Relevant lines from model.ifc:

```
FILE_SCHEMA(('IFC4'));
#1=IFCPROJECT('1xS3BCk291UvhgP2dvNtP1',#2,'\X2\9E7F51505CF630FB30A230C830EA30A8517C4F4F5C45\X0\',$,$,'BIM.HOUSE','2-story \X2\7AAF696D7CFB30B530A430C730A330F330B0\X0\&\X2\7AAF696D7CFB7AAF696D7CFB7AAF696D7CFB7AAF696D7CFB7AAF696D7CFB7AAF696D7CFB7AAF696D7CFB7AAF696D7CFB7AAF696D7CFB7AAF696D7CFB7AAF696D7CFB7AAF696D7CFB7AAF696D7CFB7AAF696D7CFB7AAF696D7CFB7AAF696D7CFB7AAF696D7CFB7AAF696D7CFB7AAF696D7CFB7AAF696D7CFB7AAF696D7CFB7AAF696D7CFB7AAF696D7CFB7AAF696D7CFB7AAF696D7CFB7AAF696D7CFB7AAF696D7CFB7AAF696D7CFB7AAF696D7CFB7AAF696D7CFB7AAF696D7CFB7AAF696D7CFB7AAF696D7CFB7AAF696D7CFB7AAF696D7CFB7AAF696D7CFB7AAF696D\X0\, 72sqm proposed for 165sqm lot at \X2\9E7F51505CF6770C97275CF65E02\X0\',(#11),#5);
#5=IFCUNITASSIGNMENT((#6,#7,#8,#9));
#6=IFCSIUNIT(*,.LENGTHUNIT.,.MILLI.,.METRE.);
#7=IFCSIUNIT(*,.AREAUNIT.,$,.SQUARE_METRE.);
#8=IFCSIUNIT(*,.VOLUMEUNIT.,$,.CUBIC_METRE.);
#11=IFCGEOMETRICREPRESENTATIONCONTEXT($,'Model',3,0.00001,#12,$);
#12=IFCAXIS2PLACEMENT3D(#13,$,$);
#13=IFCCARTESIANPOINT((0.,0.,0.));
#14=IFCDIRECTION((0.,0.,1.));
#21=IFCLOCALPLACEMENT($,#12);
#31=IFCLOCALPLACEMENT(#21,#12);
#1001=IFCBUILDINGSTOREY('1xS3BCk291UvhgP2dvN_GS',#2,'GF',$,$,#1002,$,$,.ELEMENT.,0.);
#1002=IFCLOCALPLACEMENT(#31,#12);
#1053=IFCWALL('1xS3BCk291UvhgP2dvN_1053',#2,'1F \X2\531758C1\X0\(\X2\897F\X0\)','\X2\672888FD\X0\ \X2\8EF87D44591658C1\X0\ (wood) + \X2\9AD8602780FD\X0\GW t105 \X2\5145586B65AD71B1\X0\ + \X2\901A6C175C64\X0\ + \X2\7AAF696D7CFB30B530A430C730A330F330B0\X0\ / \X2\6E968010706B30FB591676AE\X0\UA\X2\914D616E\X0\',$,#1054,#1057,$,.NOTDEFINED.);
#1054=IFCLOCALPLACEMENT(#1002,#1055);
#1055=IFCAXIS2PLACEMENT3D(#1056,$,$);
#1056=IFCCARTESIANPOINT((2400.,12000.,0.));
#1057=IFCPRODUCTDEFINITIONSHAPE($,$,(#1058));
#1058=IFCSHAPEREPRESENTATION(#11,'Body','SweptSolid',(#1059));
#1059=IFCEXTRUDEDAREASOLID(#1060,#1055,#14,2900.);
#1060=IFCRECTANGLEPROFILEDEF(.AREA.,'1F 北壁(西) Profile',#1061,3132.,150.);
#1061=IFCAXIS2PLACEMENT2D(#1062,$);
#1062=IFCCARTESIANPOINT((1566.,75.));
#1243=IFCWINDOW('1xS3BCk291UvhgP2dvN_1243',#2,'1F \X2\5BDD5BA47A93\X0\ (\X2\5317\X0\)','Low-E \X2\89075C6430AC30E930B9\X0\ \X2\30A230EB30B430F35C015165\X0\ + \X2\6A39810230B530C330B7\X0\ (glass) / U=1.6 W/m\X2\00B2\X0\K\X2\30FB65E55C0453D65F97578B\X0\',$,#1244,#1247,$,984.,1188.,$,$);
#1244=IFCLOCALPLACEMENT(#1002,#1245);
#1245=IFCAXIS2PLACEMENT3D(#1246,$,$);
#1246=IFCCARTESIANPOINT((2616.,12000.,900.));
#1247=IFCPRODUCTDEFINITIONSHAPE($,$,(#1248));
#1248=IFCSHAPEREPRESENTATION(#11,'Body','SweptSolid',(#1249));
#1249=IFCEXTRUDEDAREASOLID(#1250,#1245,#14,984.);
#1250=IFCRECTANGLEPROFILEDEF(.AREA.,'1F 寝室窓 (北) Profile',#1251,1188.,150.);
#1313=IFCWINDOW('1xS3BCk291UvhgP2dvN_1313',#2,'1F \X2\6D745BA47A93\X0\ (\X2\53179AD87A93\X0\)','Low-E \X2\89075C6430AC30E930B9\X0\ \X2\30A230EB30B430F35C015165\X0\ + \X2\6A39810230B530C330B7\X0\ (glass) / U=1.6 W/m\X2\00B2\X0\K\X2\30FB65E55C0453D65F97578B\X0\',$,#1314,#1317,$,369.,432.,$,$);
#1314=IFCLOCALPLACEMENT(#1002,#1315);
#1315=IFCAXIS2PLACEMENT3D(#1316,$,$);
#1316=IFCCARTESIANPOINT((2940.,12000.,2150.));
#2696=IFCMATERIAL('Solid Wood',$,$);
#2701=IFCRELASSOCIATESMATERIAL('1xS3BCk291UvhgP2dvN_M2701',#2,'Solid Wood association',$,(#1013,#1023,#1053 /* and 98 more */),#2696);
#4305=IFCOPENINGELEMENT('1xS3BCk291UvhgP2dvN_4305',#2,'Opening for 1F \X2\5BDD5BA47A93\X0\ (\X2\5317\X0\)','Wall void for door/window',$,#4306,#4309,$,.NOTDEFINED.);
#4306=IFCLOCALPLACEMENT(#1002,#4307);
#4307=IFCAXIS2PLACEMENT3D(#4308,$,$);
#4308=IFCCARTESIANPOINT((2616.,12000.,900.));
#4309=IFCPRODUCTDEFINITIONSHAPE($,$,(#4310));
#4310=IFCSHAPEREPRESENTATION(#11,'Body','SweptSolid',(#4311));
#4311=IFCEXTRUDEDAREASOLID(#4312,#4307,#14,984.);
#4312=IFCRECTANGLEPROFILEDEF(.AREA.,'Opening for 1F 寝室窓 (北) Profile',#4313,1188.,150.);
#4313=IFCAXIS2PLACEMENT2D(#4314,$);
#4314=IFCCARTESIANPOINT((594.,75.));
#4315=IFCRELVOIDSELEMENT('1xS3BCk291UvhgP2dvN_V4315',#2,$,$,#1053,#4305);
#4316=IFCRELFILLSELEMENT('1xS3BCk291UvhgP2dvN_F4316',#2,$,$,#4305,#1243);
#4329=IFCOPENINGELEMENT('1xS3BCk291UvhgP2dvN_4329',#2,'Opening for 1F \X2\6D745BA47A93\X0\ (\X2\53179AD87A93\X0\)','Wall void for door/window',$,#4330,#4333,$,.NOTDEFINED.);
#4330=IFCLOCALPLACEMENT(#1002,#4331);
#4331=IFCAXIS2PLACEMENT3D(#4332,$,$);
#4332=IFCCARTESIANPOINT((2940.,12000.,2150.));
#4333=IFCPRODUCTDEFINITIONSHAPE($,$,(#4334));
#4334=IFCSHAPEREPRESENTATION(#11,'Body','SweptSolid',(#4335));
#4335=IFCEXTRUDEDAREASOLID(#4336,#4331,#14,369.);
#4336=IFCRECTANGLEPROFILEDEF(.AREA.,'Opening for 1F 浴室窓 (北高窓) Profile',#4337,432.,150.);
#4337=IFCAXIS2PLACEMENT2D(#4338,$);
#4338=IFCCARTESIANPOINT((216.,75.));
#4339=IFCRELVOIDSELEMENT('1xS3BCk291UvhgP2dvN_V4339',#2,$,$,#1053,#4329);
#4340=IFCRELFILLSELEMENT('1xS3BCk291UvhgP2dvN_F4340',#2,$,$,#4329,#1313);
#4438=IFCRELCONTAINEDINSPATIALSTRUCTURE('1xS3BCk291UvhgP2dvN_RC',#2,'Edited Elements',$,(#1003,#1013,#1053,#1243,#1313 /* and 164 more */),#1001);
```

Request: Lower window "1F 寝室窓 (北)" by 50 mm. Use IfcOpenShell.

```python
import numpy as np
import ifcopenshell
import ifcopenshell.api.geometry
import ifcopenshell.util.placement
import ifcopenshell.util.unit

model = ifcopenshell.open("model.ifc")
unit_scale = ifcopenshell.util.unit.calculate_unit_scale(model)

window = model.by_guid("1xS3BCk291UvhgP2dvN_1243")
opening = window.FillsVoids[0].RelatingOpeningElement
dz = -0.05 / unit_scale

shift = np.array([0.0, 0.0, dz])
# The window is not placed relative to its opening, so move both.
for product in (opening, window):
    matrix = ifcopenshell.util.placement.get_local_placement(product.ObjectPlacement)
    matrix[:3, 3] += shift
    ifcopenshell.api.geometry.edit_object_placement(model, product=product, matrix=matrix, is_si=False)

print(f"moved by {dz * unit_scale:+.3f} m")

model.write("model_v2.ifc")
```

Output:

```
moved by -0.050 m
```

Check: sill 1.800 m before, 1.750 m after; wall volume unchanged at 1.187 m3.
